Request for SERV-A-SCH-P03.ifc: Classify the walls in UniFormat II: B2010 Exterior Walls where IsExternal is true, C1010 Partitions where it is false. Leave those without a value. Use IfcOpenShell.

First a look at what the model holds.

```python
import ifcopenshell
import ifcopenshell.util.element

model = ifcopenshell.open("SERV-A-SCH-P03.ifc")
print(model.schema)
print("classifications:", [c.Name for c in model.by_type("IfcClassification")])
values = [ifcopenshell.util.element.get_pset(e, "Pset_WallCommon", "IsExternal") for e in model.by_type("IfcWall")]
for value in (True, False, None):
    print("IsExternal", value, values.count(value))
```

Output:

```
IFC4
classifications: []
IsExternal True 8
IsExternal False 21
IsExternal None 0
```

```python
import ifcopenshell
import ifcopenshell.api.classification
import ifcopenshell.util.element

model = ifcopenshell.open("SERV-A-SCH-P03.ifc")

system = ifcopenshell.api.classification.add_classification(model, classification="UniFormat II")

walls = model.by_type("IfcWall")
external = {e: ifcopenshell.util.element.get_pset(e, "Pset_WallCommon", "IsExternal") for e in walls}
for flag, code, name in ((True, "B2010", "Exterior Walls"), (False, "C1010", "Partitions")):
    products = [e for e in walls if external[e] is flag]
    ifcopenshell.api.classification.add_reference(
        model, products=products, classification=system, identification=code, name=name
    )
    print(code, len(products))

model.write("SERV-A-SCH-P03_v2.ifc")
```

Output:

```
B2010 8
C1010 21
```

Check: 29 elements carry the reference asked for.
